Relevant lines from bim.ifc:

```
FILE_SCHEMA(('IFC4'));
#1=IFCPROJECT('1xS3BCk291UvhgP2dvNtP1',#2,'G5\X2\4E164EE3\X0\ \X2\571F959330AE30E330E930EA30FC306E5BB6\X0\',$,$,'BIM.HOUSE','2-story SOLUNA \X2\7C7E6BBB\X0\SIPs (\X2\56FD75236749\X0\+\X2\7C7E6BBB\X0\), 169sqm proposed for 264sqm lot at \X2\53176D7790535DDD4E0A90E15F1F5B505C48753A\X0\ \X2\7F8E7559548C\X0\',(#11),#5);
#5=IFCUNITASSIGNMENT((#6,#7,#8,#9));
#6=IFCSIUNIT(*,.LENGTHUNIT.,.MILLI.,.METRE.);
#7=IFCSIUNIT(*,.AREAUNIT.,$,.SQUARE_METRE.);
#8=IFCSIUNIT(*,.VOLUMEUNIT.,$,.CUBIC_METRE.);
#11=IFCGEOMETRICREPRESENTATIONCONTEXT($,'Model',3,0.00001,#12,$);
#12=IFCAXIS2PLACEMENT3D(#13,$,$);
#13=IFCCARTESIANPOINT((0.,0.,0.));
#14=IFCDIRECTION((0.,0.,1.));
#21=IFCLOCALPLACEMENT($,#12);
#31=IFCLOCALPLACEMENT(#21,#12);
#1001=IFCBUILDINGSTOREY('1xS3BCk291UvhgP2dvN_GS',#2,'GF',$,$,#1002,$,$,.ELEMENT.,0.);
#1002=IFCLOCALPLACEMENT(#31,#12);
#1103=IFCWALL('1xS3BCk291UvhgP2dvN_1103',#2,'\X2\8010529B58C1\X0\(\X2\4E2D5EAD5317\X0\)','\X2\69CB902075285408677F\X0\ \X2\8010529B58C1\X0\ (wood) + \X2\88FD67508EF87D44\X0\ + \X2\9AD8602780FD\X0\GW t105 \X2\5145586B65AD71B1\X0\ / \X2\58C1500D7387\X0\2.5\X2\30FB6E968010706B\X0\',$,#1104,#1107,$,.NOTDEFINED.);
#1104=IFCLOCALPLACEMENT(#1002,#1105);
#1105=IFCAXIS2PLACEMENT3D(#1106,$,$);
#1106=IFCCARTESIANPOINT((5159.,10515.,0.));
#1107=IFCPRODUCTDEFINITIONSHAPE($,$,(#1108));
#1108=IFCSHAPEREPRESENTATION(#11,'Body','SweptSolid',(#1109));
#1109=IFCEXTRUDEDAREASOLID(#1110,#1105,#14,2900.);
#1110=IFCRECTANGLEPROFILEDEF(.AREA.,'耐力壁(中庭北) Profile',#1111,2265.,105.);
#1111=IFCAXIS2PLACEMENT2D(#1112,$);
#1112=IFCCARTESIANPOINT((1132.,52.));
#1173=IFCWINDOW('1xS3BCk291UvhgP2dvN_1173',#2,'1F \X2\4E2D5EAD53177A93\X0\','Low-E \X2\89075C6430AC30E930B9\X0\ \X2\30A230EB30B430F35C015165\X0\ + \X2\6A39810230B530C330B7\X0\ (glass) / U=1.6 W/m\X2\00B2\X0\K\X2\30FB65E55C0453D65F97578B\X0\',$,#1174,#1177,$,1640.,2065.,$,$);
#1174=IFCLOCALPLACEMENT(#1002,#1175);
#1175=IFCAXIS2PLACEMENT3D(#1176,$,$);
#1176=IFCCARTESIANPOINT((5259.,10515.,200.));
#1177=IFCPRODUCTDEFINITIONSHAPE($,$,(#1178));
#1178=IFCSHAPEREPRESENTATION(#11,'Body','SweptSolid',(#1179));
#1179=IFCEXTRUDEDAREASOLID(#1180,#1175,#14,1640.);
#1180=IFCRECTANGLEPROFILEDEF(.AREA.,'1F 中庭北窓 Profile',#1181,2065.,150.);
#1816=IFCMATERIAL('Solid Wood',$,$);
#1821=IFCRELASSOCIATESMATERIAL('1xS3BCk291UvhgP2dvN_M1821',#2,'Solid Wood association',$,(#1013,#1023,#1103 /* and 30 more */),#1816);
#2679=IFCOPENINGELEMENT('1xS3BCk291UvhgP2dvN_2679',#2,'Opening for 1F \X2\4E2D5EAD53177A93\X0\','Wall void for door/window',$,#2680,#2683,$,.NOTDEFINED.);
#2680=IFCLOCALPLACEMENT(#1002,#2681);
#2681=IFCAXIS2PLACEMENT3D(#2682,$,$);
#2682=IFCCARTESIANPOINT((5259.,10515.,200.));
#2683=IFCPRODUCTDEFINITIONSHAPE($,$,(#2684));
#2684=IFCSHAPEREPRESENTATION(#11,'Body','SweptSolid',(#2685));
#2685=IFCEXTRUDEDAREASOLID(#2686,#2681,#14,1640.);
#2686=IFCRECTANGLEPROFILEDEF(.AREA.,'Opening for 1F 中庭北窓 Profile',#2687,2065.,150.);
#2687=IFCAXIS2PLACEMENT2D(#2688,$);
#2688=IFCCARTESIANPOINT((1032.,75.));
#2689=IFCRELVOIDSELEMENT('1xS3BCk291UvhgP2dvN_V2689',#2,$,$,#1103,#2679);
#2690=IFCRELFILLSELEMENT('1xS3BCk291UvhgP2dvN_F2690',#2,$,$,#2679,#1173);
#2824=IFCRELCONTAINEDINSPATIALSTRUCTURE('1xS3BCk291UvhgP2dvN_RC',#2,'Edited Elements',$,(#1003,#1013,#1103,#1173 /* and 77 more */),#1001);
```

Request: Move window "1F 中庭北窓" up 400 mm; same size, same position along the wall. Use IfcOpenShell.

```python
import numpy as np
import ifcopenshell
import ifcopenshell.api.geometry
import ifcopenshell.util.placement
import ifcopenshell.util.unit

model = ifcopenshell.open("bim.ifc")
unit_scale = ifcopenshell.util.unit.calculate_unit_scale(model)

window = model.by_guid("1xS3BCk291UvhgP2dvN_1173")
opening = window.FillsVoids[0].RelatingOpeningElement
dz = 400.0

shift = np.array([0.0, 0.0, dz])
# The window is not placed relative to its opening, so move both.
for product in (opening, window):
    matrix = ifcopenshell.util.placement.get_local_placement(product.ObjectPlacement)
    matrix[:3, 3] += shift
    ifcopenshell.api.geometry.edit_object_placement(model, product=product, matrix=matrix, is_si=False)

print(f"moved by {dz * unit_scale:+.3f} m")

model.write("bim-out.ifc")
```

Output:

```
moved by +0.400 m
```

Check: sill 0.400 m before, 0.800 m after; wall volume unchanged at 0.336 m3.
